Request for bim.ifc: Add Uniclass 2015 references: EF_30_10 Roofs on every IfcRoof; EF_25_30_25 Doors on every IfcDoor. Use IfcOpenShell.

First a look at what the model holds.

```python
import ifcopenshell

model = ifcopenshell.open("bim.ifc")
print(model.schema)
print("classifications:", [c.Name for c in model.by_type("IfcClassification")])
for ifc_class in ("IfcDoor", "IfcRoof", "IfcStair", "IfcWall", "IfcWindow"):
    print(ifc_class, len(model.by_type(ifc_class)))
```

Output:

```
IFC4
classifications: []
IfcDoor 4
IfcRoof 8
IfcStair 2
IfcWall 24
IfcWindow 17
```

```python
import ifcopenshell
import ifcopenshell.api.classification

model = ifcopenshell.open("bim.ifc")

system = ifcopenshell.api.classification.add_classification(model, classification="Uniclass 2015")

codes = {
    "IfcRoof": ("EF_30_10", "Roofs"),
    "IfcDoor": ("EF_25_30_25", "Doors"),
}
for ifc_class, (code, name) in codes.items():
    products = model.by_type(ifc_class)
    ifcopenshell.api.classification.add_reference(
        model, products=products, classification=system, identification=code, name=name
    )
    print(code, len(products))

model.write("bim_edited.ifc")
```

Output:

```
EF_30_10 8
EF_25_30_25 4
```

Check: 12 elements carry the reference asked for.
